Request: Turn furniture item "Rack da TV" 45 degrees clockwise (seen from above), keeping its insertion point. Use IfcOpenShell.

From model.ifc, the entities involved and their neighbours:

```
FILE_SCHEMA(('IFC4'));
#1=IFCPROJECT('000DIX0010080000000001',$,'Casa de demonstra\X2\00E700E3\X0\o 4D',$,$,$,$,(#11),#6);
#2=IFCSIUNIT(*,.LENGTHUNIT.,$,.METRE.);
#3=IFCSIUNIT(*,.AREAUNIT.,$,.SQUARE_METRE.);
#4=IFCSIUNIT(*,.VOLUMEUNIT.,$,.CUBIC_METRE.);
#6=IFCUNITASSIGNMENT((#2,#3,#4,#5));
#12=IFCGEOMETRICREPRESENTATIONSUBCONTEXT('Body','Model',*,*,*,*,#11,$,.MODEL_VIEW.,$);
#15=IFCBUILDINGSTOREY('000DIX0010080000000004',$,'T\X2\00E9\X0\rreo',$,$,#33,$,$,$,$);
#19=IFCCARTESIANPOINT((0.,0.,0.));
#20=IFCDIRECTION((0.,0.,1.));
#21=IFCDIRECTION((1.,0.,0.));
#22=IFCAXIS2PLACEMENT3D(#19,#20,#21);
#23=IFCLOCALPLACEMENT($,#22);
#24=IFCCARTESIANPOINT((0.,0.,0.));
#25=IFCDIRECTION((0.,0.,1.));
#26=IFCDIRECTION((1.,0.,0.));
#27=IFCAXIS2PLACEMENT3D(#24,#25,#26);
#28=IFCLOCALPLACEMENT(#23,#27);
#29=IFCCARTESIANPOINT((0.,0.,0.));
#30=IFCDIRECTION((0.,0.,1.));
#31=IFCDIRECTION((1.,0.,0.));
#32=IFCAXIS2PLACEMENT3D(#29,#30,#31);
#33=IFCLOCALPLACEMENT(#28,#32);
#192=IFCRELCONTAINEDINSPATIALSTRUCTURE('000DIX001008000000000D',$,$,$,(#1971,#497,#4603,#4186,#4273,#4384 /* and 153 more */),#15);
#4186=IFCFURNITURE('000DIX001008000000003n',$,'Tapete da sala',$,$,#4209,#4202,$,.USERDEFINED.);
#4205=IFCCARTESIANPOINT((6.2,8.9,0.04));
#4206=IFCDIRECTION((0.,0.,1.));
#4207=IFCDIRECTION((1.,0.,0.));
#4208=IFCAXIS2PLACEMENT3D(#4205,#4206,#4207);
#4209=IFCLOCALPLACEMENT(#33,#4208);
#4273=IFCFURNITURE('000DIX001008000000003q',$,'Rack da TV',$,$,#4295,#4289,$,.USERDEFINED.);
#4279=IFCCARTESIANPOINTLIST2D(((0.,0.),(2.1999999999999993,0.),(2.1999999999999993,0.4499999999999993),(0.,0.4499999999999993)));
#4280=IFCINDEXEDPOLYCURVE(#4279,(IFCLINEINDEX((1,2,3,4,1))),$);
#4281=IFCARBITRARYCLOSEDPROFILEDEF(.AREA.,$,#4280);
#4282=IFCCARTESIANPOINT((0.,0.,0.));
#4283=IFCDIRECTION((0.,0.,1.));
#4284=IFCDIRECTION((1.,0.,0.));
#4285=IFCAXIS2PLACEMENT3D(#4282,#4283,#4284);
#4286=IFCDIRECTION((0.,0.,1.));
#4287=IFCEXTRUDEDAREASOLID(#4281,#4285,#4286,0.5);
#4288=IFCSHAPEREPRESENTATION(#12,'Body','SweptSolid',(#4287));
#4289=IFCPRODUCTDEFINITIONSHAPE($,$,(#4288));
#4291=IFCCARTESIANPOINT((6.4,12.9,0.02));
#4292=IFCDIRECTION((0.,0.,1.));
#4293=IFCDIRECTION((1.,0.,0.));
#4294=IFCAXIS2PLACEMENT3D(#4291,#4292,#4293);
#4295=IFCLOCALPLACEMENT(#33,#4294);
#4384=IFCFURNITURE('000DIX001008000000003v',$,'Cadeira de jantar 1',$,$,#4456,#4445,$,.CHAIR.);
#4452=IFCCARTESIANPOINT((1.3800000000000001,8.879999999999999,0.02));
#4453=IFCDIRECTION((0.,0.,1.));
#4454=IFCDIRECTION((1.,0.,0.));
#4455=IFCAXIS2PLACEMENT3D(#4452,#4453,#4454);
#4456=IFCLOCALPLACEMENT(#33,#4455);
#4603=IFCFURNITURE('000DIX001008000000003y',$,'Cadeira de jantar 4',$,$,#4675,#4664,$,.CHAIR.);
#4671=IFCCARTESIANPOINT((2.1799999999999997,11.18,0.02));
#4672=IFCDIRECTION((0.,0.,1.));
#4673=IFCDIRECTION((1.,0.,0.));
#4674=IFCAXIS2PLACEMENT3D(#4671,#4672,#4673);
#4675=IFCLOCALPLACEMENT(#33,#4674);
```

```python
import ifcopenshell
import ifcopenshell.api.geometry
import ifcopenshell.util.placement

model = ifcopenshell.open("model.ifc")

item = model.by_guid("000DIX001008000000003q")
matrix = ifcopenshell.util.placement.get_local_placement(item.ObjectPlacement)
matrix = matrix @ ifcopenshell.util.placement.rotation(-45, "Z")
ifcopenshell.api.geometry.edit_object_placement(model, product=item, matrix=matrix, is_si=False)

print(ifcopenshell.util.placement.get_local_placement(item.ObjectPlacement).round(3) + 0.0)

model.write("model_edited.ifc")
```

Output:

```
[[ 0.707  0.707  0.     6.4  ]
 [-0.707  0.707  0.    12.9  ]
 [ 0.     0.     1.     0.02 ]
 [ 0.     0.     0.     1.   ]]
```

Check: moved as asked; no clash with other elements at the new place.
